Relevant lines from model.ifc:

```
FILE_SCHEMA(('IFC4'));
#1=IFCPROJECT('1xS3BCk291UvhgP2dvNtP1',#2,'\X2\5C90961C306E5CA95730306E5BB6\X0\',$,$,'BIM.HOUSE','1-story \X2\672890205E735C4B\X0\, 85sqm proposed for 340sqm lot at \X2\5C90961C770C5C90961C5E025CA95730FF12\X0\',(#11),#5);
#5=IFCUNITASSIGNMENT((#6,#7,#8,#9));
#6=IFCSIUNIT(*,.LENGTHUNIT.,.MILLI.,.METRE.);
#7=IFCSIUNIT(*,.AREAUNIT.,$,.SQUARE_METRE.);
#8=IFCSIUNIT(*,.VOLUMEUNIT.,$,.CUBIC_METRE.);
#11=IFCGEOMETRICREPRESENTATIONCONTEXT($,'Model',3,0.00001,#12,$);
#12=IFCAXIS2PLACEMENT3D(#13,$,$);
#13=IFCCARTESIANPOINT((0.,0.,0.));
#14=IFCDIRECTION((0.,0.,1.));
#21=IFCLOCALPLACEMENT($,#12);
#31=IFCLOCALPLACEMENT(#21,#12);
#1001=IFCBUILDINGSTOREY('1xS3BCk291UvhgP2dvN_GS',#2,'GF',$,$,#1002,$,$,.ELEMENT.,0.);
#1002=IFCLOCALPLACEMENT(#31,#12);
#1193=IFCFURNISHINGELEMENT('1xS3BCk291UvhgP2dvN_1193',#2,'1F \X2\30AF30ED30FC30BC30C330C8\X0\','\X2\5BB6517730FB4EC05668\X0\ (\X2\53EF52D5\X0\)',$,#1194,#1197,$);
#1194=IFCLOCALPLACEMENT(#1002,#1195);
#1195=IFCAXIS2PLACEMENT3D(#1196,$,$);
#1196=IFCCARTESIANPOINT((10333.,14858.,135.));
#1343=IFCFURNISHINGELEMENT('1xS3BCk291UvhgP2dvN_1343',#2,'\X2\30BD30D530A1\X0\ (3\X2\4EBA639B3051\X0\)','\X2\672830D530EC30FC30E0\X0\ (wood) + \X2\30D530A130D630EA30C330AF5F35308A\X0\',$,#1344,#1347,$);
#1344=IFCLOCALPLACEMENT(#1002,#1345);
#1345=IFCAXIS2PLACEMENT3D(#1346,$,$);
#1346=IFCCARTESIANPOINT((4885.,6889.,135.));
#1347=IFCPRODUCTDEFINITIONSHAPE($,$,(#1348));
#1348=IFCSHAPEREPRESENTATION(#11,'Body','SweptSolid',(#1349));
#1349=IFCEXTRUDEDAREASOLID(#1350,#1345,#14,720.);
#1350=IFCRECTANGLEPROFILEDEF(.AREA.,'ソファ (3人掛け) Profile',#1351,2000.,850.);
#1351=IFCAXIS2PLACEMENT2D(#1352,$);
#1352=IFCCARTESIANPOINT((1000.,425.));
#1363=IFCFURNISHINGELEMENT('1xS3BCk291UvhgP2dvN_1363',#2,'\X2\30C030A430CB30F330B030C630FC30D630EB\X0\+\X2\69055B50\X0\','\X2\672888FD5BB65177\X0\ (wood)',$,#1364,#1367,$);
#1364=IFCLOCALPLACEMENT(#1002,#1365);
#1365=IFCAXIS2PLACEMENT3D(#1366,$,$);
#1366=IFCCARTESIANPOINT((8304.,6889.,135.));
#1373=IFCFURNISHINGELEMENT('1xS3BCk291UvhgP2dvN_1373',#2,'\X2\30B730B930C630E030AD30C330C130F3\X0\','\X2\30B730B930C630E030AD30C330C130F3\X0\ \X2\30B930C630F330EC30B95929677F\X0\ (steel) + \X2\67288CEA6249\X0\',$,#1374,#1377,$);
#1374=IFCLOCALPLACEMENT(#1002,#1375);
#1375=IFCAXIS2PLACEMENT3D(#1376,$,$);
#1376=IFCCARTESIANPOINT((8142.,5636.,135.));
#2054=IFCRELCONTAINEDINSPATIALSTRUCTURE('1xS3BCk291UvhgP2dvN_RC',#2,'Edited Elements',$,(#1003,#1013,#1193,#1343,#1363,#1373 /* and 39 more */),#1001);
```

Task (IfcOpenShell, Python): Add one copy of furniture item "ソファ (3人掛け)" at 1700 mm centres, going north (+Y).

```python
import numpy as np
import ifcopenshell
import ifcopenshell.api.geometry
import ifcopenshell.api.root
import ifcopenshell.util.element
import ifcopenshell.util.placement
import ifcopenshell.util.unit

model = ifcopenshell.open("model.ifc")
unit_scale = ifcopenshell.util.unit.calculate_unit_scale(model)


def reuse_history(source, copy):
    """copy_class also copies each property set's owner history, people and application; keep the originals."""
    for rel in copy.IsDefinedBy:
        if rel.is_a("IfcRelDefinesByProperties") and (history := rel.RelatingPropertyDefinition.OwnerHistory):
            rel.RelatingPropertyDefinition.OwnerHistory = source.OwnerHistory
            ifcopenshell.util.element.remove_deep2(model, history)


source = model.by_guid("1xS3BCk291UvhgP2dvN_1343")
base = ifcopenshell.util.placement.get_local_placement(source.ObjectPlacement)
step = np.array([0.0, 1.0, 0.0]) * 1.7 / unit_scale

for i in range(1, 2):
    copy = ifcopenshell.api.root.copy_class(model, product=source)
    copy.Representation = ifcopenshell.util.element.copy_deep(
        model, source.Representation, exclude=["IfcGeometricRepresentationContext", "IfcRepresentationMap"]
    )
    reuse_history(source, copy)
    matrix = base.copy()
    matrix[:3, 3] += i * step
    print("added at", matrix[:3, 3].round(3) + 0.0)
    ifcopenshell.api.geometry.edit_object_placement(model, product=copy, matrix=matrix, is_si=False)

model.write("model_rev.ifc")
```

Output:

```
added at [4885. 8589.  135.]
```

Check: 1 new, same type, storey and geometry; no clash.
